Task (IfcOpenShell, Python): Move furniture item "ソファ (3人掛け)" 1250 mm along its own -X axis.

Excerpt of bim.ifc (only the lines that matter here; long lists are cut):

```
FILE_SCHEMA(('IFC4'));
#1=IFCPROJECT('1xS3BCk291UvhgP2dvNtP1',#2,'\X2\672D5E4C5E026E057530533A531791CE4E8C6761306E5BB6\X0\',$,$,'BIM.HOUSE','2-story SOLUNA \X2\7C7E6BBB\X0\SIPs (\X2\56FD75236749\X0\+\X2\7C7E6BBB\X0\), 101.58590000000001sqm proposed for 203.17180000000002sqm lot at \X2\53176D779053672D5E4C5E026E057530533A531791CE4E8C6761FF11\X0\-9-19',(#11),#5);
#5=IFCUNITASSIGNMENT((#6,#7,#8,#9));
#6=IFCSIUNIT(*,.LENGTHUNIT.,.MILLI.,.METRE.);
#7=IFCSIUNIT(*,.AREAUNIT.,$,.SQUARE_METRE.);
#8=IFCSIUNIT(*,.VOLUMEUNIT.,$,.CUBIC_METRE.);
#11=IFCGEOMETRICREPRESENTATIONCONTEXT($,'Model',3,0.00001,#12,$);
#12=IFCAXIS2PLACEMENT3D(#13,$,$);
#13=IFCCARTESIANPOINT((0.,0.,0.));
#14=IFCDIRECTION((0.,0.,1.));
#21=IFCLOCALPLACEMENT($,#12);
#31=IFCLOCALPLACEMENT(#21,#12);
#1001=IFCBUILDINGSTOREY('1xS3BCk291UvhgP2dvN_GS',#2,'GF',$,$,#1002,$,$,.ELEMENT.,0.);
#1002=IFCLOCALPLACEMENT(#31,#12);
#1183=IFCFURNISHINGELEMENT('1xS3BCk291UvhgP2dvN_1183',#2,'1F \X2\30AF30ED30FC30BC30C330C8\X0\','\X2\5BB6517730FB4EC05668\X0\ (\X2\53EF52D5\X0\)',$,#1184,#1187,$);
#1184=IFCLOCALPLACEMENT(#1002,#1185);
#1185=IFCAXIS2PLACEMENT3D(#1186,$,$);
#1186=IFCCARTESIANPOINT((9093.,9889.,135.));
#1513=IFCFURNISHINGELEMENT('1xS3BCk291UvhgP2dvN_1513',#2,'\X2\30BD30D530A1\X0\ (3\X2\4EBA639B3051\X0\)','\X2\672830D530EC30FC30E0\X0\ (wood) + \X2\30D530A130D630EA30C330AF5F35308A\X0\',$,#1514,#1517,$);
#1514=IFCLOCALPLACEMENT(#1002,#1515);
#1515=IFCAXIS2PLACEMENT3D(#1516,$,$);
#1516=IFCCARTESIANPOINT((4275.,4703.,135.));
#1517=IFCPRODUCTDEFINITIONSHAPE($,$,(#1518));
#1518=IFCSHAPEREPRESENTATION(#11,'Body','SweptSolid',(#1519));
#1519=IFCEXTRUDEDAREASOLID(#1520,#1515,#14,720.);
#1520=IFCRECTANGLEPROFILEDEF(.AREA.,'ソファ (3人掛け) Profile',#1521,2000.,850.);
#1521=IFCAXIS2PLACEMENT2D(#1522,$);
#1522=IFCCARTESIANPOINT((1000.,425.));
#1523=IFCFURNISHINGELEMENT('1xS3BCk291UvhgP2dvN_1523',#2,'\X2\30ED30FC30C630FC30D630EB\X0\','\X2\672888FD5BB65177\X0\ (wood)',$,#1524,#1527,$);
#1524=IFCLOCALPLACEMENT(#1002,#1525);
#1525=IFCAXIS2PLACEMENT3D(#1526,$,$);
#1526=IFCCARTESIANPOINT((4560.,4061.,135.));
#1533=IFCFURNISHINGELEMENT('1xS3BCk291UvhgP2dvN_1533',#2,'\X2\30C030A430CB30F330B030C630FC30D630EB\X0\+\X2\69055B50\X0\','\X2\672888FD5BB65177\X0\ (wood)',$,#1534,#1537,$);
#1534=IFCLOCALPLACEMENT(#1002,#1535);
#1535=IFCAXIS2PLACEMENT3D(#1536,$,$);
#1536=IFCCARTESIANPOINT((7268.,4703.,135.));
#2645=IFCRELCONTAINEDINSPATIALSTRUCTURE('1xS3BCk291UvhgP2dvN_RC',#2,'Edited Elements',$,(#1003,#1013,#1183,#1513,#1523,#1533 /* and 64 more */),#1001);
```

```python
import ifcopenshell
import ifcopenshell.api.geometry
import ifcopenshell.util.placement

model = ifcopenshell.open("bim.ifc")

item = model.by_id(1513)
matrix = ifcopenshell.util.placement.get_local_placement(item.ObjectPlacement)
matrix[:3, 3] -= matrix[:3, 0] * 1250.0
ifcopenshell.api.geometry.edit_object_placement(model, product=item, matrix=matrix, is_si=False)

print(ifcopenshell.util.placement.get_local_placement(item.ObjectPlacement).round(3) + 0.0)

model.write("bim-out.ifc")
```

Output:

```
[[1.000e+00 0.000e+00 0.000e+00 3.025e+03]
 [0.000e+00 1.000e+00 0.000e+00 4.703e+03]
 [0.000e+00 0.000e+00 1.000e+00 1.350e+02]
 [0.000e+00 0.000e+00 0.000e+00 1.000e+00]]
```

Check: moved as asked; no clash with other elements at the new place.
